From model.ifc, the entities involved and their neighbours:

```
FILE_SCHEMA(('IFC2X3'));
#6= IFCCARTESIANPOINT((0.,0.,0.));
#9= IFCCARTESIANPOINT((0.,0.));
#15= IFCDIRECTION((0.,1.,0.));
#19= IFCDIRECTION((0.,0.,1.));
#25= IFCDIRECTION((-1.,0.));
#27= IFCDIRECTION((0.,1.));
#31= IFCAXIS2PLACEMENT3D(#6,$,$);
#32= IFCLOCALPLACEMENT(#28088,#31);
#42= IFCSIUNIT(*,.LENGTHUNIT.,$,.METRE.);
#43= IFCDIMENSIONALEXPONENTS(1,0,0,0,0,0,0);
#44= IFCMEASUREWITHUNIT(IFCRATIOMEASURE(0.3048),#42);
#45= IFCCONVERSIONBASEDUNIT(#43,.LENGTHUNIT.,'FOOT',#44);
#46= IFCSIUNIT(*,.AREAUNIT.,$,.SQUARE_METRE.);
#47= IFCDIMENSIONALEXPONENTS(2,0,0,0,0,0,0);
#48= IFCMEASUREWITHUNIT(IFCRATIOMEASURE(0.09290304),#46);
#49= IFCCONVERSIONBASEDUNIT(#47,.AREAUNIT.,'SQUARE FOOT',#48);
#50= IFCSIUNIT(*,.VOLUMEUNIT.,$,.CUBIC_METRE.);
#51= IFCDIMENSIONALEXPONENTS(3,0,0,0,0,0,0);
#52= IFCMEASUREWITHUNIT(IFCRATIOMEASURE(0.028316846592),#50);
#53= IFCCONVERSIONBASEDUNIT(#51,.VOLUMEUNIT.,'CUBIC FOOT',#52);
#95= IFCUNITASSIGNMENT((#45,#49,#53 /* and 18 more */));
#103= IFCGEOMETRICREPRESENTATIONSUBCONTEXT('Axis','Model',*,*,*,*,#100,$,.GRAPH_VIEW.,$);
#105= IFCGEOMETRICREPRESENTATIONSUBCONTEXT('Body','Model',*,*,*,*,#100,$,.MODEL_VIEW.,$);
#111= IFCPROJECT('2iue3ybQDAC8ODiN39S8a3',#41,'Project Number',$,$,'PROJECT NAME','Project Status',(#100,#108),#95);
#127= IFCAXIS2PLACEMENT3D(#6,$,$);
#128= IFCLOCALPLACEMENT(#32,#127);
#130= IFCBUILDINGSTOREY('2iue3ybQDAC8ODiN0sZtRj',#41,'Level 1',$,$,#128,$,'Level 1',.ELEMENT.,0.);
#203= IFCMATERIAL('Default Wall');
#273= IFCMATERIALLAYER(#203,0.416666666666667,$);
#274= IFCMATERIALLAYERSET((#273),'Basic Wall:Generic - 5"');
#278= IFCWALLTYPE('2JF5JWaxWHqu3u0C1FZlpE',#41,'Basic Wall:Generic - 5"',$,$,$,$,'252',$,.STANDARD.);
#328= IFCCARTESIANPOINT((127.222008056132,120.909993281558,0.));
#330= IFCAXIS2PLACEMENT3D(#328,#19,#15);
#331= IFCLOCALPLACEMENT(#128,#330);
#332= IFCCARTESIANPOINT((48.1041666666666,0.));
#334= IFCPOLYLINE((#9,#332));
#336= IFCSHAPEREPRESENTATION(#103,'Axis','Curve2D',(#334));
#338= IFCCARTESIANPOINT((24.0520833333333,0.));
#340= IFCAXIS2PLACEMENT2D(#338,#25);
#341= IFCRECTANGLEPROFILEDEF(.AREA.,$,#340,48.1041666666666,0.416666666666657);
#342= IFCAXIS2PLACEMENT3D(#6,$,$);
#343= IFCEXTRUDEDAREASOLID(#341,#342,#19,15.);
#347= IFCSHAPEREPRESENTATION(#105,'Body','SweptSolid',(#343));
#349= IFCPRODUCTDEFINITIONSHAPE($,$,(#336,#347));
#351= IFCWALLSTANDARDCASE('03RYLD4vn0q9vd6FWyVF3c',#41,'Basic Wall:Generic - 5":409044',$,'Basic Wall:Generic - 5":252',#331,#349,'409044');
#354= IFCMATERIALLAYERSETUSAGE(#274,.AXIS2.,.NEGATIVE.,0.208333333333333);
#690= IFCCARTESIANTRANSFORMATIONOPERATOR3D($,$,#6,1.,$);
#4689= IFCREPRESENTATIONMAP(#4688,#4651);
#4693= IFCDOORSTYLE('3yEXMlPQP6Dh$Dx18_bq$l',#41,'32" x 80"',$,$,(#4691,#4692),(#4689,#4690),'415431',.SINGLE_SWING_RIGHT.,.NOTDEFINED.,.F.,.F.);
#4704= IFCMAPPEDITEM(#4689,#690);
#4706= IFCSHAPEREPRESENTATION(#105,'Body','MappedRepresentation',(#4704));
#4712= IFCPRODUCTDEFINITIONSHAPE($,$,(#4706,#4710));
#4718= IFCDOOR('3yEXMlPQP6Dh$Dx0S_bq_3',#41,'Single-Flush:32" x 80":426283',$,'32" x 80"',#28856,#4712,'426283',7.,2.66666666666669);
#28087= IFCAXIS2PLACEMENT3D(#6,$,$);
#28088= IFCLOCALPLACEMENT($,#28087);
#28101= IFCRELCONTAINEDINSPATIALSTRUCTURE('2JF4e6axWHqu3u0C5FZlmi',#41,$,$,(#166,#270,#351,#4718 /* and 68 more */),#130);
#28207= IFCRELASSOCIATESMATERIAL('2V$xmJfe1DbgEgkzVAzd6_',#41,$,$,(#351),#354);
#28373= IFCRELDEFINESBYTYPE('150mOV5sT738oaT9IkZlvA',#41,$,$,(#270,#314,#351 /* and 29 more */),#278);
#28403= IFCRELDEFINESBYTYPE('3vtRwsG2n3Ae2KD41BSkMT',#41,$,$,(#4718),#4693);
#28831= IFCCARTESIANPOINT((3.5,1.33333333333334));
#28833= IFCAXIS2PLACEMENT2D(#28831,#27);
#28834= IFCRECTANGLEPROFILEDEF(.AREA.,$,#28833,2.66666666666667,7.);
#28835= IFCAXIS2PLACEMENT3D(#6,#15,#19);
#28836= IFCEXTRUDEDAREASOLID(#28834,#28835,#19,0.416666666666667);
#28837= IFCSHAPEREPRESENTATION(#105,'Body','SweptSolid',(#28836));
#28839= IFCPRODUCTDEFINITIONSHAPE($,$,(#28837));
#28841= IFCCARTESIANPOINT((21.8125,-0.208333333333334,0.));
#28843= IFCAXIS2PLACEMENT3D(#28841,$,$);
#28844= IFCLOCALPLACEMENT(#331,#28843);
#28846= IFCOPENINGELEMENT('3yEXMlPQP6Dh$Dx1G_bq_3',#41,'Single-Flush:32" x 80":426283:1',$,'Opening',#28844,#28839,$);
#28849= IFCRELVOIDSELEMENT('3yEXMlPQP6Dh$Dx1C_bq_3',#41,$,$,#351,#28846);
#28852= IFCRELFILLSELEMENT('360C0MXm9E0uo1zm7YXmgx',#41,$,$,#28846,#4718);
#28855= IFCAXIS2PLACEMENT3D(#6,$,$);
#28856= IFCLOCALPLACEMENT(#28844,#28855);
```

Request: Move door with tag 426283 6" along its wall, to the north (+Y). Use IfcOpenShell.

```python
import ifcopenshell
import ifcopenshell.api.geometry
import ifcopenshell.util.placement
import ifcopenshell.util.unit

model = ifcopenshell.open("model.ifc")
unit_scale = ifcopenshell.util.unit.calculate_unit_scale(model)

door = model.by_guid("3yEXMlPQP6Dh$Dx0S_bq_3")
opening = door.FillsVoids[0].RelatingOpeningElement
wall = opening.VoidsElements[0].RelatingBuildingElement

wall_matrix = ifcopenshell.util.placement.get_local_placement(wall.ObjectPlacement)
shift = wall_matrix[:3, 0] * 6 * 0.0254 / unit_scale
before = ifcopenshell.util.placement.get_local_placement(door.ObjectPlacement)[:3, 3].copy()

# The door is placed relative to its opening, so it follows when the opening moves.
matrix = ifcopenshell.util.placement.get_local_placement(opening.ObjectPlacement)
matrix[:3, 3] += shift
ifcopenshell.api.geometry.edit_object_placement(
    model, product=opening, matrix=matrix, is_si=False, should_transform_children=True
)

after = ifcopenshell.util.placement.get_local_placement(door.ObjectPlacement)[:3, 3]
print("door moved by", (after - before).round(3) + 0.0)

model.write("model-out.ifc")
```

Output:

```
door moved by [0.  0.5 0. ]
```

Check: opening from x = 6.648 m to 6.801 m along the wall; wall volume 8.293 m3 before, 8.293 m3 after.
